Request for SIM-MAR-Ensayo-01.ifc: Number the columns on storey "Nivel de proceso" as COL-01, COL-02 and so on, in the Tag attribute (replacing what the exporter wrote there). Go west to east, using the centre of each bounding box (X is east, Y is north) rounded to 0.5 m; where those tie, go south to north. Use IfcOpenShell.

First a look at what the model holds.

```python
import ifcopenshell
import ifcopenshell.util.element
import ifcopenshell.util.placement

model = ifcopenshell.open("SIM-MAR-Ensayo-01.ifc")
print(model.schema)
storey = next(s for s in model.by_type("IfcBuildingStorey") if s.Name == "Nivel de proceso")
columns = [e for e in ifcopenshell.util.element.get_decomposition(storey) if e.is_a("IfcColumn")]
for e in sorted(columns, key=lambda e: e.id()):
    origin = ifcopenshell.util.placement.get_local_placement(e.ObjectPlacement)[:3, 3]
    print(e.id(), e.Tag, e.Name, origin.round(2) + 0.0, sep=" | ")
```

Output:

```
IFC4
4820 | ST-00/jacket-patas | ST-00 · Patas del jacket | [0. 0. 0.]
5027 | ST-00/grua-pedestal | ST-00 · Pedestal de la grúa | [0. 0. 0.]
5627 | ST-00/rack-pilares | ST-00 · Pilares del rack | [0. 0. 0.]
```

```python
import ifcopenshell
import ifcopenshell.geom
import ifcopenshell.util.element
import ifcopenshell.util.shape

model = ifcopenshell.open("SIM-MAR-Ensayo-01.ifc")
settings = ifcopenshell.geom.settings()
settings.set("use-world-coords", True)


def centre(element):
    shape = ifcopenshell.geom.create_shape(settings, element)
    return ifcopenshell.util.shape.get_bbox_centroid(shape.geometry)


storey = next(s for s in model.by_type("IfcBuildingStorey") if s.Name == "Nivel de proceso")
columns = [e for e in ifcopenshell.util.element.get_decomposition(storey) if e.is_a("IfcColumn")]

# Insertion points can sit at a corner or the storey origin, so sort by the geometry (in metres).
centres = {e: centre(e) for e in columns}
columns.sort(key=lambda e: (round(centres[e][0] / 0.5), centres[e][1]))

for i, e in enumerate(columns, start=1):
    number = f"COL-{i:02d}"
    e.Tag = number
    print(e.id(), number)

model.write("SIM-MAR-Ensayo-01-out.ifc")
```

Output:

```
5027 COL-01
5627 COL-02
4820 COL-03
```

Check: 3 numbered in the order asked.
